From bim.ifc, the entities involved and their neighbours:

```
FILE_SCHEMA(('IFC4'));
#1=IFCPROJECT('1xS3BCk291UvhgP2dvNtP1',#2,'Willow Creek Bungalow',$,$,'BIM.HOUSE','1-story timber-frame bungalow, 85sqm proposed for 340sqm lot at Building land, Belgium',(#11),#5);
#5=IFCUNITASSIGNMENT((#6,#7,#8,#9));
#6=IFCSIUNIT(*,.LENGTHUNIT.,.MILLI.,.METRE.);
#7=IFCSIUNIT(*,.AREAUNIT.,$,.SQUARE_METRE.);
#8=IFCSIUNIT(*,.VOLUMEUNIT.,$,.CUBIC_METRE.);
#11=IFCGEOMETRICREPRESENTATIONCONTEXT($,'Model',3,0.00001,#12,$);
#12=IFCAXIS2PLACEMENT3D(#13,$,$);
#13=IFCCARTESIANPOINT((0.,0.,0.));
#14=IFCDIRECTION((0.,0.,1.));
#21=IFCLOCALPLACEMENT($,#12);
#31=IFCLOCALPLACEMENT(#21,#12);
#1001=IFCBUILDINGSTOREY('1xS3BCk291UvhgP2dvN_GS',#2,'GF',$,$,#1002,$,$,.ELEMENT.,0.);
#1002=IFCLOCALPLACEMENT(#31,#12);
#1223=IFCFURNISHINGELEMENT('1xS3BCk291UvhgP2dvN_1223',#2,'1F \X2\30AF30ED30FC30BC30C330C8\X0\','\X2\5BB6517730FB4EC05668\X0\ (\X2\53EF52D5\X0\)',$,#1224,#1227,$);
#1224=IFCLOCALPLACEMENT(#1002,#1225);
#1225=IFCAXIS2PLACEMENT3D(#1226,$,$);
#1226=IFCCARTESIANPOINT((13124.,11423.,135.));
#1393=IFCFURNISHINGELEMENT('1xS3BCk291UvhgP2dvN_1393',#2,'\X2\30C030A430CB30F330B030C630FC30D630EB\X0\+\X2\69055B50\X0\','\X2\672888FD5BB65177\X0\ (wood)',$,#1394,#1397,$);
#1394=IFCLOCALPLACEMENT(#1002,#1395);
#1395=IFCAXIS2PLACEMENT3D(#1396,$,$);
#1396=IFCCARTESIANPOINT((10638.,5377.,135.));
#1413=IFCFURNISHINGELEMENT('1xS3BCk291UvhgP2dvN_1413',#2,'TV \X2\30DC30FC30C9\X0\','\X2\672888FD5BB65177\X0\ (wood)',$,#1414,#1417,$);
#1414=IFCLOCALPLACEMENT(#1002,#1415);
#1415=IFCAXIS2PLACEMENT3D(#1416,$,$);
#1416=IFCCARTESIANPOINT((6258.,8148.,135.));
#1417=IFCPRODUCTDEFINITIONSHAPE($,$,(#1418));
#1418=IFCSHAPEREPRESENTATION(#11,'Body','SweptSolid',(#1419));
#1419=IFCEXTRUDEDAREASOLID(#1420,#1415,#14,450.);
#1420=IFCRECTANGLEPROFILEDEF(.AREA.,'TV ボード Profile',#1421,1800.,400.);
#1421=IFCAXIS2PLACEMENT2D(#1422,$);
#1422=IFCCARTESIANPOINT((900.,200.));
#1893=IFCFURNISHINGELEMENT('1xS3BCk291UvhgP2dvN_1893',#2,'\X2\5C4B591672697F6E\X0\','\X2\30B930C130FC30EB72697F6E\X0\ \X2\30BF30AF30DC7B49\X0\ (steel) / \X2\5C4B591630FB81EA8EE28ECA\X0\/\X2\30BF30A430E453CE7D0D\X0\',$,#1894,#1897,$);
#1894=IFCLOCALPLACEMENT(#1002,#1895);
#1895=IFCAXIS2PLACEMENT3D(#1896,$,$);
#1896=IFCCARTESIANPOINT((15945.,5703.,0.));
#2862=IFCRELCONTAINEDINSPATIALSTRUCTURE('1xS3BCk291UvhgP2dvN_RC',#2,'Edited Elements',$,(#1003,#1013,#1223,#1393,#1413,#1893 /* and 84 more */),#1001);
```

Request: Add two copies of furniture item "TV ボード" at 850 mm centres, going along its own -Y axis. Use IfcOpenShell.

```python
import ifcopenshell
import ifcopenshell.api.geometry
import ifcopenshell.api.root
import ifcopenshell.util.element
import ifcopenshell.util.placement
import ifcopenshell.util.unit

model = ifcopenshell.open("bim.ifc")
unit_scale = ifcopenshell.util.unit.calculate_unit_scale(model)


def reuse_history(source, copy):
    """copy_class also copies each property set's owner history, people and application; keep the originals."""
    for rel in copy.IsDefinedBy:
        if rel.is_a("IfcRelDefinesByProperties") and (history := rel.RelatingPropertyDefinition.OwnerHistory):
            rel.RelatingPropertyDefinition.OwnerHistory = source.OwnerHistory
            ifcopenshell.util.element.remove_deep2(model, history)


source = model.by_guid("1xS3BCk291UvhgP2dvN_1413")
base = ifcopenshell.util.placement.get_local_placement(source.ObjectPlacement)
step = -base[:3, 1] * 0.85 / unit_scale

for i in range(1, 3):
    copy = ifcopenshell.api.root.copy_class(model, product=source)
    copy.Representation = ifcopenshell.util.element.copy_deep(
        model, source.Representation, exclude=["IfcGeometricRepresentationContext", "IfcRepresentationMap"]
    )
    reuse_history(source, copy)
    matrix = base.copy()
    matrix[:3, 3] += i * step
    print("added at", matrix[:3, 3].round(3) + 0.0)
    ifcopenshell.api.geometry.edit_object_placement(model, product=copy, matrix=matrix, is_si=False)

model.write("bim_edited.ifc")
```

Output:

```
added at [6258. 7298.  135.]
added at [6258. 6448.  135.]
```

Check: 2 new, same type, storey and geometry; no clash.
